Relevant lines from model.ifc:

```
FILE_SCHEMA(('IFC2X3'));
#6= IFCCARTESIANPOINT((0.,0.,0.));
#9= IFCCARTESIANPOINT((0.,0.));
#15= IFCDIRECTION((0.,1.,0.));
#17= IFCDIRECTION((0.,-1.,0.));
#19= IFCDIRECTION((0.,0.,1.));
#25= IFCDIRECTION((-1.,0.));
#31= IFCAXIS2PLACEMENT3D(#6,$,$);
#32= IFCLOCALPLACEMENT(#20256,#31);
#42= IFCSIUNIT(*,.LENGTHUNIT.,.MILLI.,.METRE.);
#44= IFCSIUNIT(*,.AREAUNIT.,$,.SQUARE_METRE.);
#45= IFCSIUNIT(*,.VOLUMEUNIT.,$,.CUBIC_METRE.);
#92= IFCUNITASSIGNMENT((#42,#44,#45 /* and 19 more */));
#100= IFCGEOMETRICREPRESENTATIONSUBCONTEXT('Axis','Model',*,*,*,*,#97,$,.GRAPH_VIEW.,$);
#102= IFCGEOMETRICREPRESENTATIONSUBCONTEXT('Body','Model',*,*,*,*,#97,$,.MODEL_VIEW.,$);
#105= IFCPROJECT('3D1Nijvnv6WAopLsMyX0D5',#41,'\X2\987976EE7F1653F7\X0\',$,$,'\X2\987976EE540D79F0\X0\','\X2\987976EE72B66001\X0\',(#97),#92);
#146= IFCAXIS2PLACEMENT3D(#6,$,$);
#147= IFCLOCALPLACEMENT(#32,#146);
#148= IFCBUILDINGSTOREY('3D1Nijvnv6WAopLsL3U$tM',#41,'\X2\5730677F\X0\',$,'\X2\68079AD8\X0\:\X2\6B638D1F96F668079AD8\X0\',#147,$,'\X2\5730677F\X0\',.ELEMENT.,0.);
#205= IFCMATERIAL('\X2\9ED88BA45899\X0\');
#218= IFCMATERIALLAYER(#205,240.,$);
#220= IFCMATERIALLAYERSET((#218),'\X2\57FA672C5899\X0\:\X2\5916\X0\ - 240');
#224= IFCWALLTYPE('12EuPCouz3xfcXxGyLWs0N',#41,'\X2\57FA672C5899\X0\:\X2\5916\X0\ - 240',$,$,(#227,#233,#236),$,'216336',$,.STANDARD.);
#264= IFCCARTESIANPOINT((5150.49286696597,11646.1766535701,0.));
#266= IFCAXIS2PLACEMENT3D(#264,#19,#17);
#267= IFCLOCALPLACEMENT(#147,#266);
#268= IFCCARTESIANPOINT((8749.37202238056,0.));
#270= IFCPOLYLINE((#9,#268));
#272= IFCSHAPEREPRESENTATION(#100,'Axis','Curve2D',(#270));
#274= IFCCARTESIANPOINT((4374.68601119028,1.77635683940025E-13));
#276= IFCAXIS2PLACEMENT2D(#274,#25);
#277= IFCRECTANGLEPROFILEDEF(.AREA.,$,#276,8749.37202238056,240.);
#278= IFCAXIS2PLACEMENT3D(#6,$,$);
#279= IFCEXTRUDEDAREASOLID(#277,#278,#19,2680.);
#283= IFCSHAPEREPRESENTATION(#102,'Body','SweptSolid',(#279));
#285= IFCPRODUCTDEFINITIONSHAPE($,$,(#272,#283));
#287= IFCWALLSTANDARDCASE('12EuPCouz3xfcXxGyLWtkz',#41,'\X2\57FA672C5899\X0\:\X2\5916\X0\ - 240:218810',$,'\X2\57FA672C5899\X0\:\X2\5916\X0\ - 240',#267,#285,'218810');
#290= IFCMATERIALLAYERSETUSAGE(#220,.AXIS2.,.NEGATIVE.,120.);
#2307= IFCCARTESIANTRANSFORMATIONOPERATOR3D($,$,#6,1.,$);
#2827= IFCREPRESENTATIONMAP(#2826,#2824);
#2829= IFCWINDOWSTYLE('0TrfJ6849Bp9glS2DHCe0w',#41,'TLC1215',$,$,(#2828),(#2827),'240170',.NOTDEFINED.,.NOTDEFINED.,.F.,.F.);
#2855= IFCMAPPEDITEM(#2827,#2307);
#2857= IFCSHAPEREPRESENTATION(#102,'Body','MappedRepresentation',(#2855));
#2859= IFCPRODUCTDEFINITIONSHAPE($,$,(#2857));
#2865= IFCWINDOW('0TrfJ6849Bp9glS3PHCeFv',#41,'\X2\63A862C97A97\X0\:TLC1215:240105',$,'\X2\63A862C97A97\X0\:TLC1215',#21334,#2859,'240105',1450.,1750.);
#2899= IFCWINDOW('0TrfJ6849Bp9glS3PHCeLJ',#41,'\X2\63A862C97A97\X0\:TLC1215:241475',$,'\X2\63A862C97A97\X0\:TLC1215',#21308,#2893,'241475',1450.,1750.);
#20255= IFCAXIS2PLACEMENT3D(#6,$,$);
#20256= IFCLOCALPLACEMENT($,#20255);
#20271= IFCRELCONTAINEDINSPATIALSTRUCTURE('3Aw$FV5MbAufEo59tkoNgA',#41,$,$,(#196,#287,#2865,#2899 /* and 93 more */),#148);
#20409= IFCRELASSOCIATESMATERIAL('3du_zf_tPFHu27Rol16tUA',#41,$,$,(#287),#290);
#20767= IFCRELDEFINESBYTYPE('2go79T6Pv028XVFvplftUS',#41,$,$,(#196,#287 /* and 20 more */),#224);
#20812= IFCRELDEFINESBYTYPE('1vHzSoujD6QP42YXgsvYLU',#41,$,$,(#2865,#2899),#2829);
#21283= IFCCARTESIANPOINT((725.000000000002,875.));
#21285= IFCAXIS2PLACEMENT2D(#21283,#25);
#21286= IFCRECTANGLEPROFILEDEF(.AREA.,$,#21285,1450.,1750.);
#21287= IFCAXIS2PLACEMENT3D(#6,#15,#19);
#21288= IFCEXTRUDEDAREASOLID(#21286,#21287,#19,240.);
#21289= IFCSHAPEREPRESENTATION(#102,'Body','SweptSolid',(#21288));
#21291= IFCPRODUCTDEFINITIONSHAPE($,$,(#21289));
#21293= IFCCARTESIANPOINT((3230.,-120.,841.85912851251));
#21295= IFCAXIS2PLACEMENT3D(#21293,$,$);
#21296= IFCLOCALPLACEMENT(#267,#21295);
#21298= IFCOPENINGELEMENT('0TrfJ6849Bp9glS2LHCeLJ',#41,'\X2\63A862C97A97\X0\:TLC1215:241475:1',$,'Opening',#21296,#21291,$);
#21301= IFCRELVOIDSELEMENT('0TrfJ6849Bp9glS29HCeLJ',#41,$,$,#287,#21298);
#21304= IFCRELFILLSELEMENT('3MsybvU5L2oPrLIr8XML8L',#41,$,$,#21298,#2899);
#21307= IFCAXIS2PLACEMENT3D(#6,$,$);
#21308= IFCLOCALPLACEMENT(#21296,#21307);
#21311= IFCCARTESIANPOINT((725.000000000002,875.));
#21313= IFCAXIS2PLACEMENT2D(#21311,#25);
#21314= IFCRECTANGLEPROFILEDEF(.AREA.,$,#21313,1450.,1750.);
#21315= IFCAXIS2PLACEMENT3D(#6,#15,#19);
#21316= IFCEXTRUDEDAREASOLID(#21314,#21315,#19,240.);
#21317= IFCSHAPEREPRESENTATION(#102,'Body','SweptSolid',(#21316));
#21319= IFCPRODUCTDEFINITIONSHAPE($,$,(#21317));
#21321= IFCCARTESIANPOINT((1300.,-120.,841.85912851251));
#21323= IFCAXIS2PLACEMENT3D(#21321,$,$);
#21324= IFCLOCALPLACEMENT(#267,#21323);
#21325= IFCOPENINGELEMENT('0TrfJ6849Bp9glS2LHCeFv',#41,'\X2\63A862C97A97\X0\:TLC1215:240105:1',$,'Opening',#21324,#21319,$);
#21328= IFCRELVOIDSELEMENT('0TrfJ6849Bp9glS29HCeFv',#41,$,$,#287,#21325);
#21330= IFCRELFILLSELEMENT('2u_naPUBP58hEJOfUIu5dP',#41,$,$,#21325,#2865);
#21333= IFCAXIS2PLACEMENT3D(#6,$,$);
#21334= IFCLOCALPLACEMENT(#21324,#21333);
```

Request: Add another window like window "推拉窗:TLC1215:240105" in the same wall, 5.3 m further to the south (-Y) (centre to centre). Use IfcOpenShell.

```python
import ifcopenshell
import ifcopenshell.api.feature
import ifcopenshell.api.geometry
import ifcopenshell.api.root
import ifcopenshell.geom
import ifcopenshell.util.element
import ifcopenshell.util.placement
import ifcopenshell.util.shape

model = ifcopenshell.open("model.ifc")
settings = ifcopenshell.geom.settings()


def volume(element):
    """Net volume in cubic metres, openings subtracted."""
    shape = ifcopenshell.geom.create_shape(settings, element)
    return ifcopenshell.util.shape.get_volume(shape.geometry)


def reuse_history(source, copy):
    """copy_class also copies each property set's owner history, people and application; keep the originals."""
    for rel in copy.IsDefinedBy:
        if rel.is_a("IfcRelDefinesByProperties") and (history := rel.RelatingPropertyDefinition.OwnerHistory):
            rel.RelatingPropertyDefinition.OwnerHistory = source.OwnerHistory
            ifcopenshell.util.element.remove_deep2(model, history)


window = model.by_guid("0TrfJ6849Bp9glS3PHCeFv")
opening = window.FillsVoids[0].RelatingOpeningElement
wall = opening.VoidsElements[0].RelatingBuildingElement
before = volume(wall)
shift = ifcopenshell.util.placement.get_local_placement(wall.ObjectPlacement)[:3, 0] * 5300.0

# copy_class copies the void relationship, type, container and properties, but no geometry.
new_opening = ifcopenshell.api.root.copy_class(model, product=opening)
new_opening.Representation = ifcopenshell.util.element.copy_deep(
    model, opening.Representation, exclude=["IfcGeometricRepresentationContext", "IfcRepresentationMap"]
)
new_opening.Name = "推拉窗:TLC1215"
new_window = ifcopenshell.api.root.copy_class(model, product=window)
new_window.Representation = ifcopenshell.util.element.copy_deep(
    model, window.Representation, exclude=["IfcGeometricRepresentationContext", "IfcRepresentationMap"]
)
new_window.Name = "推拉窗:TLC1215"
new_window.Tag = None
reuse_history(window, new_window)
fills = ifcopenshell.api.feature.add_filling(model, opening=new_opening, element=new_window)
fills.OwnerHistory = new_window.OwnerHistory  # required in IFC2X3

for old, new in ((opening, new_opening), (window, new_window)):
    matrix = ifcopenshell.util.placement.get_local_placement(old.ObjectPlacement)
    matrix[:3, 3] += shift
    ifcopenshell.api.geometry.edit_object_placement(model, product=new, matrix=matrix, is_si=False)

after = volume(wall)

print(f"wall volume {before:.3f} -> {after:.3f} m3")

model.write("model_rev.ifc")
```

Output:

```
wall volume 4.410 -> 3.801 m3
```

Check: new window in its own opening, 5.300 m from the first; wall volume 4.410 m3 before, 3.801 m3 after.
